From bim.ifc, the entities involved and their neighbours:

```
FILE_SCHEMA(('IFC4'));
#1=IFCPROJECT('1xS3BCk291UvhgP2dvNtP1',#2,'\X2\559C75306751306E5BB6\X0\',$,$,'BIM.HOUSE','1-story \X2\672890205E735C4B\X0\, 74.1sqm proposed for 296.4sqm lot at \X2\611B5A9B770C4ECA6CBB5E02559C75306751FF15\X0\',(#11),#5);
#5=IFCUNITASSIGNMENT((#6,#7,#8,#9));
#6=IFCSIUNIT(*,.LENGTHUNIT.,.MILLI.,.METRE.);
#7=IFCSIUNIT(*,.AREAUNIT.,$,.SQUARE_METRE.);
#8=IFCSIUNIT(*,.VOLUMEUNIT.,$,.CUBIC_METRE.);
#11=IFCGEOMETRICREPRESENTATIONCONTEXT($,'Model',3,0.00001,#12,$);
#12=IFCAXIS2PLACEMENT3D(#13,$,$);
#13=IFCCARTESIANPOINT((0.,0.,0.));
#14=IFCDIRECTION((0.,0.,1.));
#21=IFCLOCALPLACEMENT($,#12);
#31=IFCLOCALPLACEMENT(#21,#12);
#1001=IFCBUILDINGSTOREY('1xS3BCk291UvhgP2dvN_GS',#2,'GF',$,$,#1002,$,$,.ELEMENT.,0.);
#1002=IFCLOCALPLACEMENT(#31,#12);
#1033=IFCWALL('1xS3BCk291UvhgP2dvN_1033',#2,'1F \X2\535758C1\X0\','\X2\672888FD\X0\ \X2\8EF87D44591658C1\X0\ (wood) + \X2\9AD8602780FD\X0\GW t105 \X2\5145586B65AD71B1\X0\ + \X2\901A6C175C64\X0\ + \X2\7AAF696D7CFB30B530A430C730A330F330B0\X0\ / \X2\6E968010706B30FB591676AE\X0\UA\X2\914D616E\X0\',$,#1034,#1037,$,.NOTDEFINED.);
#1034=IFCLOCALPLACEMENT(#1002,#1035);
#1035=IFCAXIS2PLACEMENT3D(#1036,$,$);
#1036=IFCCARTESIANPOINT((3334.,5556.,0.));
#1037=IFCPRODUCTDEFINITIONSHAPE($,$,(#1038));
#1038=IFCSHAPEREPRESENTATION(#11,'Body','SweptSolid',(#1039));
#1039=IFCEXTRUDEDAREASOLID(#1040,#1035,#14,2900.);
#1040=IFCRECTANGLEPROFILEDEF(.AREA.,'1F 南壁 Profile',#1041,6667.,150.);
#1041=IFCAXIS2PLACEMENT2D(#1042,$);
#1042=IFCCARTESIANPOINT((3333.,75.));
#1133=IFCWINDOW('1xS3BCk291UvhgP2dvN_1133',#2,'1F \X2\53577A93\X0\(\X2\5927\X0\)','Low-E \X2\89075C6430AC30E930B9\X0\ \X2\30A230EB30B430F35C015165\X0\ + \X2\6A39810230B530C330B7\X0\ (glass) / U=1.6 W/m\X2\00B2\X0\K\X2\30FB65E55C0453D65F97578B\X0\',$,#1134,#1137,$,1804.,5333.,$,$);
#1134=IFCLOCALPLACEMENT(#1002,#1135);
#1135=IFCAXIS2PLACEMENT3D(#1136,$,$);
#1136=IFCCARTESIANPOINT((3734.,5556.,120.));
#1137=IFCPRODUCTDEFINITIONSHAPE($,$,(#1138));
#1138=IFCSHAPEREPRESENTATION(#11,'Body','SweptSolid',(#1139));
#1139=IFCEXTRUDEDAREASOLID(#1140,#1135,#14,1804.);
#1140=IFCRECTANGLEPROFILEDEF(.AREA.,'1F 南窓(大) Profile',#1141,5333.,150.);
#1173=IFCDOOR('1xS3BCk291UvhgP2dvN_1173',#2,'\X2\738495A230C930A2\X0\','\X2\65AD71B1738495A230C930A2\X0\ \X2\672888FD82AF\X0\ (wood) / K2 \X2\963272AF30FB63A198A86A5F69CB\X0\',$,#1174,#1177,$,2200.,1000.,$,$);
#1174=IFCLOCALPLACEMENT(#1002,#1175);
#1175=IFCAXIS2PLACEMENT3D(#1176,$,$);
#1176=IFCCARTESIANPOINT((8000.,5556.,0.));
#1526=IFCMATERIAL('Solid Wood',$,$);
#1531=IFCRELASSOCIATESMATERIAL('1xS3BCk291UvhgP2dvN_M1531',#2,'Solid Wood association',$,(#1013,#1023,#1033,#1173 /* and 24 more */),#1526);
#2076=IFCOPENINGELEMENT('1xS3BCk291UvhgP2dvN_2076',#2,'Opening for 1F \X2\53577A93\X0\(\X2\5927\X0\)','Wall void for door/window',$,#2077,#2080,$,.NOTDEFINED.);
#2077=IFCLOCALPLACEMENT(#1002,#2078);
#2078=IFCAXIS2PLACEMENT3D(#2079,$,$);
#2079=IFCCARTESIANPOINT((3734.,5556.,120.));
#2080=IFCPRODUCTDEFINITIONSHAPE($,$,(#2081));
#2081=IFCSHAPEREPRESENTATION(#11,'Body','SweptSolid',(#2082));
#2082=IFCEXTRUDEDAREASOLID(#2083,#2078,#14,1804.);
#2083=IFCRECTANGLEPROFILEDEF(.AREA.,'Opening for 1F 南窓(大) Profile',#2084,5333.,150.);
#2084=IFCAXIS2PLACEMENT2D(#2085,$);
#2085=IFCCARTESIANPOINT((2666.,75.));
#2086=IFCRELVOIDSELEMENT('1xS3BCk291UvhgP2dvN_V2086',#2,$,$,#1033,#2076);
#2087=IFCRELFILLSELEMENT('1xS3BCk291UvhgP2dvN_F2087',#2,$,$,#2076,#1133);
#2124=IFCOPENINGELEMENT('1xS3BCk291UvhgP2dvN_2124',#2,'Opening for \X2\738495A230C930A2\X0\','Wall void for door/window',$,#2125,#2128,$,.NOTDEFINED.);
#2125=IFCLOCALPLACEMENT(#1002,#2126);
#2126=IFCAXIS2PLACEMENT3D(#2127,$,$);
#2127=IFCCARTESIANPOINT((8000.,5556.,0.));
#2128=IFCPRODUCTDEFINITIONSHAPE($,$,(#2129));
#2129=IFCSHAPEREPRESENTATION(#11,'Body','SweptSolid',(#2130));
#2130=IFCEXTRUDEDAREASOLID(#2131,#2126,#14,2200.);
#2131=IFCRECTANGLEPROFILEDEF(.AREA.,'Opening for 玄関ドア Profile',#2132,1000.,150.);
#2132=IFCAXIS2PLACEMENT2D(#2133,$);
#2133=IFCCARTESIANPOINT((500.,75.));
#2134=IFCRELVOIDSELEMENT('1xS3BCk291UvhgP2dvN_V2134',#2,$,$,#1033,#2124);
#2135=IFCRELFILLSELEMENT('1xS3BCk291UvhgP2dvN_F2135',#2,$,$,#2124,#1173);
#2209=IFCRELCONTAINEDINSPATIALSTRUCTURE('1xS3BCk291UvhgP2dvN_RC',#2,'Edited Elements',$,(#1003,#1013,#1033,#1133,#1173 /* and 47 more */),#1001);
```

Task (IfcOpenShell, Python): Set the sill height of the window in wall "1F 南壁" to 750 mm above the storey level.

```python
import numpy as np
import ifcopenshell
import ifcopenshell.api.geometry
import ifcopenshell.geom
import ifcopenshell.util.element
import ifcopenshell.util.placement
import ifcopenshell.util.shape
import ifcopenshell.util.unit

model = ifcopenshell.open("bim.ifc")
unit_scale = ifcopenshell.util.unit.calculate_unit_scale(model)

window = model.by_guid("1xS3BCk291UvhgP2dvN_1133")
opening = window.FillsVoids[0].RelatingOpeningElement
storey = ifcopenshell.util.element.get_container(window, ifc_class="IfcBuildingStorey")
level = ifcopenshell.util.placement.get_local_placement(storey.ObjectPlacement)[2, 3]

# The opening's origin need not be at the sill, so measure its lowest point.
shape = ifcopenshell.geom.create_shape(ifcopenshell.geom.settings(), opening)
bottom = ifcopenshell.util.shape.get_shape_bottom_elevation(shape, shape.geometry) / unit_scale
dz = level + 0.75 / unit_scale - bottom

shift = np.array([0.0, 0.0, dz])
# The window is not placed relative to its opening, so move both.
for product in (opening, window):
    matrix = ifcopenshell.util.placement.get_local_placement(product.ObjectPlacement)
    matrix[:3, 3] += shift
    ifcopenshell.api.geometry.edit_object_placement(model, product=product, matrix=matrix, is_si=False)

print(f"moved by {dz * unit_scale:+.3f} m")

model.write("bim_edited.ifc")
```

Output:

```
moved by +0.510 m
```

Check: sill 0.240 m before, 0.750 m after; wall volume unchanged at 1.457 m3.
